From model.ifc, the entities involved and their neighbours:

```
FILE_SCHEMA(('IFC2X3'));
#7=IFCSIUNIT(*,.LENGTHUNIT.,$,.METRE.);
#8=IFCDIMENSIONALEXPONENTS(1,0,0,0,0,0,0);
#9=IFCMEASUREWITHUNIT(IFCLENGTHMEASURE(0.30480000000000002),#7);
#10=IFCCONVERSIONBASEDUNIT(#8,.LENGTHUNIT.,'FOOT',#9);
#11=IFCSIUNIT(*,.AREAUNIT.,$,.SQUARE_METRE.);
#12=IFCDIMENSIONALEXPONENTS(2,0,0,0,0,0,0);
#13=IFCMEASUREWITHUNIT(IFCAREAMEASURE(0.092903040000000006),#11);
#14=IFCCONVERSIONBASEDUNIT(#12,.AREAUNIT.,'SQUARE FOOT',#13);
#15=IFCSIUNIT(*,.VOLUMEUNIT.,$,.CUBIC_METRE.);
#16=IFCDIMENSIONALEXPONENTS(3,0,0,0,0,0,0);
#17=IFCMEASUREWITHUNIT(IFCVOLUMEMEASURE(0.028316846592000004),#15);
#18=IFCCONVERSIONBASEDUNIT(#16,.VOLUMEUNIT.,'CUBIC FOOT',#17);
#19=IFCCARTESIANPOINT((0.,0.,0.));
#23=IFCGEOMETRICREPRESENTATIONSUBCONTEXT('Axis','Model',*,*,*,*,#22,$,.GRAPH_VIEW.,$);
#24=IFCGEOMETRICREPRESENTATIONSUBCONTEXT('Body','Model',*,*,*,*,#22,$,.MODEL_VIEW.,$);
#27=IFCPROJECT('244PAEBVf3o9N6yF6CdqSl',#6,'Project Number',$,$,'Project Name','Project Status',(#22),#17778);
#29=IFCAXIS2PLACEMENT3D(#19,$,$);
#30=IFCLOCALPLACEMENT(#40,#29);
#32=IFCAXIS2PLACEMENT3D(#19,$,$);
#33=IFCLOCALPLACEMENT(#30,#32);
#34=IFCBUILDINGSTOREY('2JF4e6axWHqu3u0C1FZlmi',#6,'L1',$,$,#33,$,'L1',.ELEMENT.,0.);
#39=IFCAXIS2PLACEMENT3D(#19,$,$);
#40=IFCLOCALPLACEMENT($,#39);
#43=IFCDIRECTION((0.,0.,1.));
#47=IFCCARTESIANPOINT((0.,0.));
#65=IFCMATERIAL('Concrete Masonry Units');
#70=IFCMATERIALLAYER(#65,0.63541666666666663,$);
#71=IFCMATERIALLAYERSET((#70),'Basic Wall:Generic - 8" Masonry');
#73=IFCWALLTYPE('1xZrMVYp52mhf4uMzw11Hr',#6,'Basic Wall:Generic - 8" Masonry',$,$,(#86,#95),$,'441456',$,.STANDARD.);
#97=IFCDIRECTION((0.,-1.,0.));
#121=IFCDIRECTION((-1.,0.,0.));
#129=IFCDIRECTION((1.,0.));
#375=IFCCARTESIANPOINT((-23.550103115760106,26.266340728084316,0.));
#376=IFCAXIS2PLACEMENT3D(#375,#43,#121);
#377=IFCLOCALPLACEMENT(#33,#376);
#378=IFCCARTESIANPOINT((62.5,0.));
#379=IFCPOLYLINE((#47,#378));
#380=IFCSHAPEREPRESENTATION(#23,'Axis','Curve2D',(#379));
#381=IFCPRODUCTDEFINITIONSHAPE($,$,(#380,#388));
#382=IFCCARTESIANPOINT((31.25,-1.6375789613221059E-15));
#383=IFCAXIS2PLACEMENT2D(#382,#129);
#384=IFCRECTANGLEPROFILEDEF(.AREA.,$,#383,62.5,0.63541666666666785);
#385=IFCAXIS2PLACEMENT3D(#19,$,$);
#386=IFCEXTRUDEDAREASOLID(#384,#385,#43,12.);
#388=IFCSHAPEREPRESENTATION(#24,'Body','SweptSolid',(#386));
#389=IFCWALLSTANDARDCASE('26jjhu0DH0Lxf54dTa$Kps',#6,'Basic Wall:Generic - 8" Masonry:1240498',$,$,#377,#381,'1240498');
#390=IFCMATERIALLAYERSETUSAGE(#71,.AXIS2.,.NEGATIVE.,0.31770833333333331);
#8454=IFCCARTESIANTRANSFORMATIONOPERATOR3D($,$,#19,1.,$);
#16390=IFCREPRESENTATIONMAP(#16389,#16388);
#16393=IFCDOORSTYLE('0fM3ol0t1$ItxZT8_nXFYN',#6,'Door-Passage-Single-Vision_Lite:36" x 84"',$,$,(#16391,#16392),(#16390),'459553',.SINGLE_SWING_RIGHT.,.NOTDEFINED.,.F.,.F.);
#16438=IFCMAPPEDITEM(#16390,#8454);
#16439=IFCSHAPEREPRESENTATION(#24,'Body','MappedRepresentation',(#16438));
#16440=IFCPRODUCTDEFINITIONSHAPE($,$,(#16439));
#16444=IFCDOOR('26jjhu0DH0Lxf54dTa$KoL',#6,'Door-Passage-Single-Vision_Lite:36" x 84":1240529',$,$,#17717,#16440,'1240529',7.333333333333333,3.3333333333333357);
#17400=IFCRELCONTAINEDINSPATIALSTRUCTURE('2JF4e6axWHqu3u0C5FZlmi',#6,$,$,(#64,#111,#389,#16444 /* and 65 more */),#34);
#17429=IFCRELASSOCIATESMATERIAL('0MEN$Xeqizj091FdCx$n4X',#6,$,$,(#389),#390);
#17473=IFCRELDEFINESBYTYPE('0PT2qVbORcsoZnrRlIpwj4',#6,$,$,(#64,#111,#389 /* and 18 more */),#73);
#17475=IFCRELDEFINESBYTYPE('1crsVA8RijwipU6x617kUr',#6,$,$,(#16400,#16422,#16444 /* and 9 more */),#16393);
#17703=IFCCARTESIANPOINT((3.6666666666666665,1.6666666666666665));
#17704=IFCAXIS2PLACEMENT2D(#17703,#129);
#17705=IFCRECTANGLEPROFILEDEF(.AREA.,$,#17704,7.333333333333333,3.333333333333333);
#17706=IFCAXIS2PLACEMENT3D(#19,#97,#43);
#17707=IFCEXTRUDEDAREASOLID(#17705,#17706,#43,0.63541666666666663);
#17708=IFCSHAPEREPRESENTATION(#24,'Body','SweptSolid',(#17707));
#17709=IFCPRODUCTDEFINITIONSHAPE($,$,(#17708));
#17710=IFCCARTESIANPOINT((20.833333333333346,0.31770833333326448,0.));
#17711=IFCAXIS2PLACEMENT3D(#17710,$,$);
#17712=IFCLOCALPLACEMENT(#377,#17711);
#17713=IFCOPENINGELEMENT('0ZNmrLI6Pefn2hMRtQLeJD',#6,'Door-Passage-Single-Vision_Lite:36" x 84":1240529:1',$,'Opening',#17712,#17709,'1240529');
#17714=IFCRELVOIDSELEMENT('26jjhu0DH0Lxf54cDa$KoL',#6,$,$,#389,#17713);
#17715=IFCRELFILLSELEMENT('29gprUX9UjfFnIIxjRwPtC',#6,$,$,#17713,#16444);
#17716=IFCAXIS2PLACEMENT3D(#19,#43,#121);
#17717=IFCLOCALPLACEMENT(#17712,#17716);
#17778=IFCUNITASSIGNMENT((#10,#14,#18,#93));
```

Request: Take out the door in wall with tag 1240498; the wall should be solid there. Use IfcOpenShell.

```python
import ifcopenshell
import ifcopenshell.api.feature
import ifcopenshell.api.root
import ifcopenshell.geom
import ifcopenshell.util.shape

model = ifcopenshell.open("model.ifc")
settings = ifcopenshell.geom.settings()


def volume(element):
    """Net volume in cubic metres, openings subtracted."""
    shape = ifcopenshell.geom.create_shape(settings, element)
    return ifcopenshell.util.shape.get_volume(shape.geometry)


door = model.by_guid("26jjhu0DH0Lxf54dTa$KoL")
opening = door.FillsVoids[0].RelatingOpeningElement
wall = opening.VoidsElements[0].RelatingBuildingElement
before = volume(wall)

ifcopenshell.api.root.remove_product(model, product=door)
ifcopenshell.api.feature.remove_feature(model, feature=opening)

after = volume(wall)

print(f"wall volume {before:.3f} -> {after:.3f} m3")

model.write("model_updated.ifc")
```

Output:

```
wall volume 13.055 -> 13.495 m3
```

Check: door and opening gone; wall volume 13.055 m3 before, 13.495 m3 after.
